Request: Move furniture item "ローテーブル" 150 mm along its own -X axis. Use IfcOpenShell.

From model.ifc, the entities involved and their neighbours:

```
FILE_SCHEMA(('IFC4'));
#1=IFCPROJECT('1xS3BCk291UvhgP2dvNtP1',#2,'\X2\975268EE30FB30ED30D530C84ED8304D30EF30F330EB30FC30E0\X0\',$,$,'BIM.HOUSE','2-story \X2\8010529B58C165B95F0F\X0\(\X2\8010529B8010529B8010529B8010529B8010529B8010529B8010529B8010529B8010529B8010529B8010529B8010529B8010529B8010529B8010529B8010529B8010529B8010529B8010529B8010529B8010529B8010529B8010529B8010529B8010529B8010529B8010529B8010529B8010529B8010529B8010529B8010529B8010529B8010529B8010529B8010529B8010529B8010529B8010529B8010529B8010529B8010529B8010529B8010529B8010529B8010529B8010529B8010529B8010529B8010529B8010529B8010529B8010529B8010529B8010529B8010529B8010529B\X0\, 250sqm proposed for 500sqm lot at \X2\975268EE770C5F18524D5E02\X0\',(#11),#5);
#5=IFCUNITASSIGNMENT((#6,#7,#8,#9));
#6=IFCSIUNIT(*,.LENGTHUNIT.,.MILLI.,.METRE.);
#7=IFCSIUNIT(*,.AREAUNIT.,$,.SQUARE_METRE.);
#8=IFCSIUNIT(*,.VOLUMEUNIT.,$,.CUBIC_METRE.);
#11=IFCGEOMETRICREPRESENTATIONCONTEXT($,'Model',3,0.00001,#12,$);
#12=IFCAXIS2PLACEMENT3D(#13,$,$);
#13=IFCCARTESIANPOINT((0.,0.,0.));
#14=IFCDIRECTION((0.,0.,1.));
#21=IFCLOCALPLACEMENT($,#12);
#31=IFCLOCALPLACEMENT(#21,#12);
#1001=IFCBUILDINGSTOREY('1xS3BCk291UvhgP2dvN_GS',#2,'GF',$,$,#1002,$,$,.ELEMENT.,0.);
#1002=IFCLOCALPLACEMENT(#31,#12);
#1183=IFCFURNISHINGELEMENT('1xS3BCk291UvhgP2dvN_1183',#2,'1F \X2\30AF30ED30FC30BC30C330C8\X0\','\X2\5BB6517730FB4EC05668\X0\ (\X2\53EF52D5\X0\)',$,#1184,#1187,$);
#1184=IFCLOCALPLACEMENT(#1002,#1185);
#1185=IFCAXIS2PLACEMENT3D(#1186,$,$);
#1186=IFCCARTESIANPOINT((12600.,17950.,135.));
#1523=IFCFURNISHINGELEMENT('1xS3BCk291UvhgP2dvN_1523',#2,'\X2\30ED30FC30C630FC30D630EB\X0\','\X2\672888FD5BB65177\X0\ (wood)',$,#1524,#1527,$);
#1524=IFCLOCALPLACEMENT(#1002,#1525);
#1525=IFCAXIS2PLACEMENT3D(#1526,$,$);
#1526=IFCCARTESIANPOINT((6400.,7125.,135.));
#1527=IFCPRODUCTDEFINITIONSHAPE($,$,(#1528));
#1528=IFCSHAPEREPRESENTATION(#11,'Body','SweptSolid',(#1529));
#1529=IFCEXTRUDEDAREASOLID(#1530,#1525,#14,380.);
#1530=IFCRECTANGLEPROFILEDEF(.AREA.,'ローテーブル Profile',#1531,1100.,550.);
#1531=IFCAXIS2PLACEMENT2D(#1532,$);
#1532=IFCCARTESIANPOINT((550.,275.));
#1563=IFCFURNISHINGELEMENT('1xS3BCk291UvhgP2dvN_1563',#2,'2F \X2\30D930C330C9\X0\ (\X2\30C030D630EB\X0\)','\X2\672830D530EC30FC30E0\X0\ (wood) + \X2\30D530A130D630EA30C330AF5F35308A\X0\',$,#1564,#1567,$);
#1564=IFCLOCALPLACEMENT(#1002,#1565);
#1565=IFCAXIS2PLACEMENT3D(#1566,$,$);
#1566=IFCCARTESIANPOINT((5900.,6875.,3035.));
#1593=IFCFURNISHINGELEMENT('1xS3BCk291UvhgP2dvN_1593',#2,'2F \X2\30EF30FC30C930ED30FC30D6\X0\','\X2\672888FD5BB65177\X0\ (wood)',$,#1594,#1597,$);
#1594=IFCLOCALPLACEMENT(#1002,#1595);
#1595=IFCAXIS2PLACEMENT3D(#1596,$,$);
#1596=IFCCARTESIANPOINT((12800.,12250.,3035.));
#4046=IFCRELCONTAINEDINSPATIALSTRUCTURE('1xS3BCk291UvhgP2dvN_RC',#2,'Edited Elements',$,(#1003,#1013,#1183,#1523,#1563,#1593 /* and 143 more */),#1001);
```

```python
import ifcopenshell
import ifcopenshell.api.geometry
import ifcopenshell.util.placement
import ifcopenshell.util.unit

model = ifcopenshell.open("model.ifc")
unit_scale = ifcopenshell.util.unit.calculate_unit_scale(model)

item = model.by_guid("1xS3BCk291UvhgP2dvN_1523")
matrix = ifcopenshell.util.placement.get_local_placement(item.ObjectPlacement)
matrix[:3, 3] -= matrix[:3, 0] * 0.15 / unit_scale
ifcopenshell.api.geometry.edit_object_placement(model, product=item, matrix=matrix, is_si=False)

print(ifcopenshell.util.placement.get_local_placement(item.ObjectPlacement).round(3) + 0.0)

model.write("model-out.ifc")
```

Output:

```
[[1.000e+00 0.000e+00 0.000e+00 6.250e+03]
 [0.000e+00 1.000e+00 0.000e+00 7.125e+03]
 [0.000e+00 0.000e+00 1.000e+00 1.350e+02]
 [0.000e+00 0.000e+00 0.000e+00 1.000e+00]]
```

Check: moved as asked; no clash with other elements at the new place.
